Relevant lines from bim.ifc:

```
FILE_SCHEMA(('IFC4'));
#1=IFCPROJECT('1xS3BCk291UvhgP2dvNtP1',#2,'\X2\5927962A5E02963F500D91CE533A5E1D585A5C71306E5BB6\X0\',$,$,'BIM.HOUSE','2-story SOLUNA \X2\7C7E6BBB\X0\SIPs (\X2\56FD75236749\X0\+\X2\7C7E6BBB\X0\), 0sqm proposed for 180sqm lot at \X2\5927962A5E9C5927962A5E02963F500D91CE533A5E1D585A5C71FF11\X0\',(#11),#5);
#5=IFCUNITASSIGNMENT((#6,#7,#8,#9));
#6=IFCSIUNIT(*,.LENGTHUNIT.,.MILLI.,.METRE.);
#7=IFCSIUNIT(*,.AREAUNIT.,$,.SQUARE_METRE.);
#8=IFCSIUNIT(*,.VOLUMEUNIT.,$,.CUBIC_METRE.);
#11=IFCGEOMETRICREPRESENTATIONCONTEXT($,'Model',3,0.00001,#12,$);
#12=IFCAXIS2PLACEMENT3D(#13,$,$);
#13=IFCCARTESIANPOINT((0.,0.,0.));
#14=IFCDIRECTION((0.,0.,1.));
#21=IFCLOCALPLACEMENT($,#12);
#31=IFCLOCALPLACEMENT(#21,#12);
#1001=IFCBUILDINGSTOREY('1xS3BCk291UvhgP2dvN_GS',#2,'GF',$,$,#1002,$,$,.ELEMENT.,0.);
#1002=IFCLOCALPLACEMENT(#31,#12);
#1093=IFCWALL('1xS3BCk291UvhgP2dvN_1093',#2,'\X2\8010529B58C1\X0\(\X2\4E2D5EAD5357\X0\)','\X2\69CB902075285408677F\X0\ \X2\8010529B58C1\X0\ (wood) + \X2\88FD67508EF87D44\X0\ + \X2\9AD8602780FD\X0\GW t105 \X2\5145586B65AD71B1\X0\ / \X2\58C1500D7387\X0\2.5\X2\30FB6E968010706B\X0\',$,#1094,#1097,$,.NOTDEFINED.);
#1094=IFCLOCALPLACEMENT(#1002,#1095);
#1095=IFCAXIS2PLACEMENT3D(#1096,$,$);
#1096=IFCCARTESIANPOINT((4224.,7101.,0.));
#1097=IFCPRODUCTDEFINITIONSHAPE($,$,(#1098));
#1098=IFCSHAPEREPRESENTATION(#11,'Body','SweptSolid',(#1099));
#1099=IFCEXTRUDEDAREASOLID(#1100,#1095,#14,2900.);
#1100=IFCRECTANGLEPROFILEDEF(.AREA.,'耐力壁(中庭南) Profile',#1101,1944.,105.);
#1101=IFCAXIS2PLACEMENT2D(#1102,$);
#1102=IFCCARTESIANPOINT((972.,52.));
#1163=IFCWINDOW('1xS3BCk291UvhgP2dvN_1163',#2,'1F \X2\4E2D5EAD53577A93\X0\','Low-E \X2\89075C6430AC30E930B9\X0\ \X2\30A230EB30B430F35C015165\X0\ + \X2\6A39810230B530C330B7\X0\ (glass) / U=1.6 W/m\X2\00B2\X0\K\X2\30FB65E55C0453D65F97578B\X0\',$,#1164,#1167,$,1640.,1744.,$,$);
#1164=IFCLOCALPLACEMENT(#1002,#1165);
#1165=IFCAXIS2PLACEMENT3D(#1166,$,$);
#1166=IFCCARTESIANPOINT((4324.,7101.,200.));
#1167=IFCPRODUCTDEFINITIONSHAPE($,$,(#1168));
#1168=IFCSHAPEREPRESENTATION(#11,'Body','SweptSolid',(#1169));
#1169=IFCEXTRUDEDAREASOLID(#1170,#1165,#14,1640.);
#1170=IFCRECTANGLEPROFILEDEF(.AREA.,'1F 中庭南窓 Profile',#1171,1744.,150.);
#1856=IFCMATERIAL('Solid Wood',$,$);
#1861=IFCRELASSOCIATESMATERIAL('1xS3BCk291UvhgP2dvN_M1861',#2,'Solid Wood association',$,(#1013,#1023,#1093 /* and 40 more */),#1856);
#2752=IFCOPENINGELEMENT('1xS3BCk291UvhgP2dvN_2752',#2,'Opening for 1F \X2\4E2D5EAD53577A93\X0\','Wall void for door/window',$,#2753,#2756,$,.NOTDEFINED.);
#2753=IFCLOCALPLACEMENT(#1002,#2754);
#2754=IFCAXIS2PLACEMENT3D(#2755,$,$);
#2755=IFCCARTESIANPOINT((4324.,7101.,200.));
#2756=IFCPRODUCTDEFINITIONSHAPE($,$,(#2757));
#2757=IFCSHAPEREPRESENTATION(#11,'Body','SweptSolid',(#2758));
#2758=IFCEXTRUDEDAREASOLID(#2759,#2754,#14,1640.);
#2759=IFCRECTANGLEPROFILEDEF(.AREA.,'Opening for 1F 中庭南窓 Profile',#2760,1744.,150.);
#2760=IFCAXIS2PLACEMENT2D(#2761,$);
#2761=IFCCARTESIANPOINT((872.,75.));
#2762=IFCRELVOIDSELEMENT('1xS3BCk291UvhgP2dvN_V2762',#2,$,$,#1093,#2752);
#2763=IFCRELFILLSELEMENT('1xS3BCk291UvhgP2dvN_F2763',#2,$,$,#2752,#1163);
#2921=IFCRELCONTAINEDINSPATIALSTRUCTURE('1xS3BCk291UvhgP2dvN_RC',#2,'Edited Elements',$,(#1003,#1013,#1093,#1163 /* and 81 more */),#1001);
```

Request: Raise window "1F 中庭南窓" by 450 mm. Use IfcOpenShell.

```python
import numpy as np
import ifcopenshell
import ifcopenshell.api.geometry
import ifcopenshell.util.placement
import ifcopenshell.util.unit

model = ifcopenshell.open("bim.ifc")
unit_scale = ifcopenshell.util.unit.calculate_unit_scale(model)

window = model.by_guid("1xS3BCk291UvhgP2dvN_1163")
opening = window.FillsVoids[0].RelatingOpeningElement
dz = 0.45 / unit_scale

shift = np.array([0.0, 0.0, dz])
# The window is not placed relative to its opening, so move both.
for product in (opening, window):
    matrix = ifcopenshell.util.placement.get_local_placement(product.ObjectPlacement)
    matrix[:3, 3] += shift
    ifcopenshell.api.geometry.edit_object_placement(model, product=product, matrix=matrix, is_si=False)

print(f"moved by {dz * unit_scale:+.3f} m")

model.write("bim_updated.ifc")
```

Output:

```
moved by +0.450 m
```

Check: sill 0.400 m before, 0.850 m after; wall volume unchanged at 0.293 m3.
